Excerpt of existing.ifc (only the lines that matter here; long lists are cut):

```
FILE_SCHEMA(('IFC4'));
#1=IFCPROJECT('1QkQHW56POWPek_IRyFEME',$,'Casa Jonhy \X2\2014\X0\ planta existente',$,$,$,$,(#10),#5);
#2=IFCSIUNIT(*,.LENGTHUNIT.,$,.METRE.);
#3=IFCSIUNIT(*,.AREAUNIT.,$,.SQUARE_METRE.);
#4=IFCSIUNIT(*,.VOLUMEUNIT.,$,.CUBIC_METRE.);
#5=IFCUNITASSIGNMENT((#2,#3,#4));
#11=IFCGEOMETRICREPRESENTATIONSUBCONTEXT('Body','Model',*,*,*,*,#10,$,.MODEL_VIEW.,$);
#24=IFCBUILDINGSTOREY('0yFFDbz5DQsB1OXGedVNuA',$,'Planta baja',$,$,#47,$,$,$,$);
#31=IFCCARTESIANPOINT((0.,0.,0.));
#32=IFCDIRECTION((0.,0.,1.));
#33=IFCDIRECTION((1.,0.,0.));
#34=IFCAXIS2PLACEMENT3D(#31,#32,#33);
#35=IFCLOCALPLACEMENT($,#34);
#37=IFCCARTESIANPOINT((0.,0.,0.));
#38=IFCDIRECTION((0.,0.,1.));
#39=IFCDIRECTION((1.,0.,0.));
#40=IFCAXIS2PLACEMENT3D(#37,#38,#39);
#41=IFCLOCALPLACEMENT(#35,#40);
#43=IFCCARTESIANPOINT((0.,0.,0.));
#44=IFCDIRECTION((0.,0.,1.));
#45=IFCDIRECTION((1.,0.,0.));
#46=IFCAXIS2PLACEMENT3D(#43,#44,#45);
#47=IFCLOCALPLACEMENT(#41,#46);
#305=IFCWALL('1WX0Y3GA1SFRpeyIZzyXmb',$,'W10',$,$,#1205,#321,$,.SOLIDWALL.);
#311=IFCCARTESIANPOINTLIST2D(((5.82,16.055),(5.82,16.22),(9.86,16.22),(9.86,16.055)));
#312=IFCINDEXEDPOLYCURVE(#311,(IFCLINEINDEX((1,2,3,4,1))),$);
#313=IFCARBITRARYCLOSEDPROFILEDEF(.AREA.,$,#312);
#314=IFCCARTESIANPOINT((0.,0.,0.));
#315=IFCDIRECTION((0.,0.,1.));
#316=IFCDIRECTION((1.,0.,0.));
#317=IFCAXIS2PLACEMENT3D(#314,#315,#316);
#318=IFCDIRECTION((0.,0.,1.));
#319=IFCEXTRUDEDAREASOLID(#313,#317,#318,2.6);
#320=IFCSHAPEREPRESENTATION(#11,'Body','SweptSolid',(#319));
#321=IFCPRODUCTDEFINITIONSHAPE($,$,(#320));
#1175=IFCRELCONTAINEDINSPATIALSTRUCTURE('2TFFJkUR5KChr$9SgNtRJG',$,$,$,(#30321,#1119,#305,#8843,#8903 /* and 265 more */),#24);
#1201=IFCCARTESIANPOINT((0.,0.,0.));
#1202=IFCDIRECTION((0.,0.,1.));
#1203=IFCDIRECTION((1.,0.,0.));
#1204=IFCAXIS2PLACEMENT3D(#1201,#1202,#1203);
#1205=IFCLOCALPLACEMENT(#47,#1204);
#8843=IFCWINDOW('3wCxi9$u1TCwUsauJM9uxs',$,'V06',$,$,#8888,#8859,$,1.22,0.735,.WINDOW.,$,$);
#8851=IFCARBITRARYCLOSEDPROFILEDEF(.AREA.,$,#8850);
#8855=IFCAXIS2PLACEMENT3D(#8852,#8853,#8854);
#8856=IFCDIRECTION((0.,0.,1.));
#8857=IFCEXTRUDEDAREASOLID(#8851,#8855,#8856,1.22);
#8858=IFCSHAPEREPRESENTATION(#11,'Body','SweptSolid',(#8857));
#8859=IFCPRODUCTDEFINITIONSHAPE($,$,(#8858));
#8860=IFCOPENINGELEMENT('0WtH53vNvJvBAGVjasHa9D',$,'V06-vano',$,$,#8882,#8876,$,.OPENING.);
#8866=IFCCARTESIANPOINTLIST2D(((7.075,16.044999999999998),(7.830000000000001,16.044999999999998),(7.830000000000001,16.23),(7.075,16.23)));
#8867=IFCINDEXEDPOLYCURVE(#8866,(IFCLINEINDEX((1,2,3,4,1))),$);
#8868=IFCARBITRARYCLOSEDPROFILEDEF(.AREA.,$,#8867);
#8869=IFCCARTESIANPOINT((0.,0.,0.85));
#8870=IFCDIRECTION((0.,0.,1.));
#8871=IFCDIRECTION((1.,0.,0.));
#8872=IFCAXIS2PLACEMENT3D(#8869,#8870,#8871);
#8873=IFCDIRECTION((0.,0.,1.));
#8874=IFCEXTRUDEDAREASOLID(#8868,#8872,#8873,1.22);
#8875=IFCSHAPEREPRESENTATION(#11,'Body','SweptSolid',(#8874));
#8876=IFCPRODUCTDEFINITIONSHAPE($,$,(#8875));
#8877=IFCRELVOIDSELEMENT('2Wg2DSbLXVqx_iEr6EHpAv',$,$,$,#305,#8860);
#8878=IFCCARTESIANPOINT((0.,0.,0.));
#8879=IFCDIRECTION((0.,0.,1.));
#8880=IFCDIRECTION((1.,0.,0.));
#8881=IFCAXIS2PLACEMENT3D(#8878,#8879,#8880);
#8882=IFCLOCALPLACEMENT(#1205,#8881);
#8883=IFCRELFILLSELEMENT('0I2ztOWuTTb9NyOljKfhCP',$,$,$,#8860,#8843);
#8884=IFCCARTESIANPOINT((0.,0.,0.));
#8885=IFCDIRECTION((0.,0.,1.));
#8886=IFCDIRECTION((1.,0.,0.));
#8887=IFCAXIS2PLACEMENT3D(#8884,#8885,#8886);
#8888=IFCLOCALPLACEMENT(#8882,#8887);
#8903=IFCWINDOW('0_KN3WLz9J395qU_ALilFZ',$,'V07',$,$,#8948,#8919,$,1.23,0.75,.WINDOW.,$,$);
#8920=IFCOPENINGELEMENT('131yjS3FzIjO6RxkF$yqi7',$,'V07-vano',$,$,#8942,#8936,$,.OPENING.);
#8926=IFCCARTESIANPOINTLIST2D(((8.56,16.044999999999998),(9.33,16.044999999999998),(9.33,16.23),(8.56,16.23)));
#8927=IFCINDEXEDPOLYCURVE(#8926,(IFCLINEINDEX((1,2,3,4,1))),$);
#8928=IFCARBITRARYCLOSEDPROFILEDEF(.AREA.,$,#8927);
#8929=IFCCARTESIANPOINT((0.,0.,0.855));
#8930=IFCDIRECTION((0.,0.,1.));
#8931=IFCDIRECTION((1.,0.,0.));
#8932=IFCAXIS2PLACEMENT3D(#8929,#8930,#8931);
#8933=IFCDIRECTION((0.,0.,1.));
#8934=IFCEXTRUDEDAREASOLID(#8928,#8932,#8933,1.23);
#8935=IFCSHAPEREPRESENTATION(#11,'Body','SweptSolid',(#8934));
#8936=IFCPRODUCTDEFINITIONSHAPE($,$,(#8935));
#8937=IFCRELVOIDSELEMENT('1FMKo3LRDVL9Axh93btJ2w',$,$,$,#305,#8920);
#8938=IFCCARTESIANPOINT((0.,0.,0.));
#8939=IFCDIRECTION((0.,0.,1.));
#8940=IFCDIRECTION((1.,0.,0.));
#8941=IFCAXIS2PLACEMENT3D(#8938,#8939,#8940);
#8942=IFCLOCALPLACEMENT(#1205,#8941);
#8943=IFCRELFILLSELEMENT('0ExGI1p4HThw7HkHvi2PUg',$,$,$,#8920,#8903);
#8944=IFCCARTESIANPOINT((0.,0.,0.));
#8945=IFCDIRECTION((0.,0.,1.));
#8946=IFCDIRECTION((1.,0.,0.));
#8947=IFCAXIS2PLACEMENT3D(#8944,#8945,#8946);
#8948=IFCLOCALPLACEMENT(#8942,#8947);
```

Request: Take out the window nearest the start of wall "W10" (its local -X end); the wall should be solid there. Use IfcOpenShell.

```python
import ifcopenshell
import ifcopenshell.api.feature
import ifcopenshell.api.root
import ifcopenshell.geom
import ifcopenshell.util.shape

model = ifcopenshell.open("existing.ifc")
settings = ifcopenshell.geom.settings()


def volume(element):
    """Net volume in cubic metres, openings subtracted."""
    shape = ifcopenshell.geom.create_shape(settings, element)
    return ifcopenshell.util.shape.get_volume(shape.geometry)


window = model.by_guid("3wCxi9$u1TCwUsauJM9uxs")
opening = window.FillsVoids[0].RelatingOpeningElement
wall = opening.VoidsElements[0].RelatingBuildingElement
before = volume(wall)

ifcopenshell.api.root.remove_product(model, product=window)
ifcopenshell.api.feature.remove_feature(model, feature=opening)

after = volume(wall)

print(f"wall volume {before:.3f} -> {after:.3f} m3")

model.write("existing_v2.ifc")
```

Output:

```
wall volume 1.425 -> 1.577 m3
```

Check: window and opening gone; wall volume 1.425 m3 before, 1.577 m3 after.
